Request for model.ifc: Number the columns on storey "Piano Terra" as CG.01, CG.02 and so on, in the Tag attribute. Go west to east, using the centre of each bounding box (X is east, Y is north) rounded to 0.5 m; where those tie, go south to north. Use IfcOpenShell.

First a look at what the model holds.

```python
import ifcopenshell
import ifcopenshell.util.element
import ifcopenshell.util.placement

model = ifcopenshell.open("model.ifc")
print(model.schema)
storey = next(s for s in model.by_type("IfcBuildingStorey") if s.Name == "Piano Terra")
columns = [e for e in ifcopenshell.util.element.get_decomposition(storey) if e.is_a("IfcColumn")]
for e in sorted(columns, key=lambda e: e.id()):
    origin = ifcopenshell.util.placement.get_local_placement(e.ObjectPlacement)[:3, 3]
    print(e.id(), e.Tag, e.Name, origin.round(2) + 0.0, sep=" | ")
```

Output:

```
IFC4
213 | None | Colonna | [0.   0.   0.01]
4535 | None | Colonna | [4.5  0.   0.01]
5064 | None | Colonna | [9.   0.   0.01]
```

```python
import ifcopenshell
import ifcopenshell.geom
import ifcopenshell.util.element
import ifcopenshell.util.shape

model = ifcopenshell.open("model.ifc")
settings = ifcopenshell.geom.settings()
settings.set("use-world-coords", True)


def centre(element):
    shape = ifcopenshell.geom.create_shape(settings, element)
    return ifcopenshell.util.shape.get_bbox_centroid(shape.geometry)


storey = next(s for s in model.by_type("IfcBuildingStorey") if s.Name == "Piano Terra")
columns = [e for e in ifcopenshell.util.element.get_decomposition(storey) if e.is_a("IfcColumn")]

# Insertion points can sit at a corner or the storey origin, so sort by the geometry (in metres).
centres = {e: centre(e) for e in columns}
columns.sort(key=lambda e: (round(centres[e][0] / 0.5), centres[e][1]))

for i, e in enumerate(columns, start=1):
    number = f"CG.{i:02d}"
    e.Tag = number
    print(e.id(), number)

model.write("model_updated.ifc")
```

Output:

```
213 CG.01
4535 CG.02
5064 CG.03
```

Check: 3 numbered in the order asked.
